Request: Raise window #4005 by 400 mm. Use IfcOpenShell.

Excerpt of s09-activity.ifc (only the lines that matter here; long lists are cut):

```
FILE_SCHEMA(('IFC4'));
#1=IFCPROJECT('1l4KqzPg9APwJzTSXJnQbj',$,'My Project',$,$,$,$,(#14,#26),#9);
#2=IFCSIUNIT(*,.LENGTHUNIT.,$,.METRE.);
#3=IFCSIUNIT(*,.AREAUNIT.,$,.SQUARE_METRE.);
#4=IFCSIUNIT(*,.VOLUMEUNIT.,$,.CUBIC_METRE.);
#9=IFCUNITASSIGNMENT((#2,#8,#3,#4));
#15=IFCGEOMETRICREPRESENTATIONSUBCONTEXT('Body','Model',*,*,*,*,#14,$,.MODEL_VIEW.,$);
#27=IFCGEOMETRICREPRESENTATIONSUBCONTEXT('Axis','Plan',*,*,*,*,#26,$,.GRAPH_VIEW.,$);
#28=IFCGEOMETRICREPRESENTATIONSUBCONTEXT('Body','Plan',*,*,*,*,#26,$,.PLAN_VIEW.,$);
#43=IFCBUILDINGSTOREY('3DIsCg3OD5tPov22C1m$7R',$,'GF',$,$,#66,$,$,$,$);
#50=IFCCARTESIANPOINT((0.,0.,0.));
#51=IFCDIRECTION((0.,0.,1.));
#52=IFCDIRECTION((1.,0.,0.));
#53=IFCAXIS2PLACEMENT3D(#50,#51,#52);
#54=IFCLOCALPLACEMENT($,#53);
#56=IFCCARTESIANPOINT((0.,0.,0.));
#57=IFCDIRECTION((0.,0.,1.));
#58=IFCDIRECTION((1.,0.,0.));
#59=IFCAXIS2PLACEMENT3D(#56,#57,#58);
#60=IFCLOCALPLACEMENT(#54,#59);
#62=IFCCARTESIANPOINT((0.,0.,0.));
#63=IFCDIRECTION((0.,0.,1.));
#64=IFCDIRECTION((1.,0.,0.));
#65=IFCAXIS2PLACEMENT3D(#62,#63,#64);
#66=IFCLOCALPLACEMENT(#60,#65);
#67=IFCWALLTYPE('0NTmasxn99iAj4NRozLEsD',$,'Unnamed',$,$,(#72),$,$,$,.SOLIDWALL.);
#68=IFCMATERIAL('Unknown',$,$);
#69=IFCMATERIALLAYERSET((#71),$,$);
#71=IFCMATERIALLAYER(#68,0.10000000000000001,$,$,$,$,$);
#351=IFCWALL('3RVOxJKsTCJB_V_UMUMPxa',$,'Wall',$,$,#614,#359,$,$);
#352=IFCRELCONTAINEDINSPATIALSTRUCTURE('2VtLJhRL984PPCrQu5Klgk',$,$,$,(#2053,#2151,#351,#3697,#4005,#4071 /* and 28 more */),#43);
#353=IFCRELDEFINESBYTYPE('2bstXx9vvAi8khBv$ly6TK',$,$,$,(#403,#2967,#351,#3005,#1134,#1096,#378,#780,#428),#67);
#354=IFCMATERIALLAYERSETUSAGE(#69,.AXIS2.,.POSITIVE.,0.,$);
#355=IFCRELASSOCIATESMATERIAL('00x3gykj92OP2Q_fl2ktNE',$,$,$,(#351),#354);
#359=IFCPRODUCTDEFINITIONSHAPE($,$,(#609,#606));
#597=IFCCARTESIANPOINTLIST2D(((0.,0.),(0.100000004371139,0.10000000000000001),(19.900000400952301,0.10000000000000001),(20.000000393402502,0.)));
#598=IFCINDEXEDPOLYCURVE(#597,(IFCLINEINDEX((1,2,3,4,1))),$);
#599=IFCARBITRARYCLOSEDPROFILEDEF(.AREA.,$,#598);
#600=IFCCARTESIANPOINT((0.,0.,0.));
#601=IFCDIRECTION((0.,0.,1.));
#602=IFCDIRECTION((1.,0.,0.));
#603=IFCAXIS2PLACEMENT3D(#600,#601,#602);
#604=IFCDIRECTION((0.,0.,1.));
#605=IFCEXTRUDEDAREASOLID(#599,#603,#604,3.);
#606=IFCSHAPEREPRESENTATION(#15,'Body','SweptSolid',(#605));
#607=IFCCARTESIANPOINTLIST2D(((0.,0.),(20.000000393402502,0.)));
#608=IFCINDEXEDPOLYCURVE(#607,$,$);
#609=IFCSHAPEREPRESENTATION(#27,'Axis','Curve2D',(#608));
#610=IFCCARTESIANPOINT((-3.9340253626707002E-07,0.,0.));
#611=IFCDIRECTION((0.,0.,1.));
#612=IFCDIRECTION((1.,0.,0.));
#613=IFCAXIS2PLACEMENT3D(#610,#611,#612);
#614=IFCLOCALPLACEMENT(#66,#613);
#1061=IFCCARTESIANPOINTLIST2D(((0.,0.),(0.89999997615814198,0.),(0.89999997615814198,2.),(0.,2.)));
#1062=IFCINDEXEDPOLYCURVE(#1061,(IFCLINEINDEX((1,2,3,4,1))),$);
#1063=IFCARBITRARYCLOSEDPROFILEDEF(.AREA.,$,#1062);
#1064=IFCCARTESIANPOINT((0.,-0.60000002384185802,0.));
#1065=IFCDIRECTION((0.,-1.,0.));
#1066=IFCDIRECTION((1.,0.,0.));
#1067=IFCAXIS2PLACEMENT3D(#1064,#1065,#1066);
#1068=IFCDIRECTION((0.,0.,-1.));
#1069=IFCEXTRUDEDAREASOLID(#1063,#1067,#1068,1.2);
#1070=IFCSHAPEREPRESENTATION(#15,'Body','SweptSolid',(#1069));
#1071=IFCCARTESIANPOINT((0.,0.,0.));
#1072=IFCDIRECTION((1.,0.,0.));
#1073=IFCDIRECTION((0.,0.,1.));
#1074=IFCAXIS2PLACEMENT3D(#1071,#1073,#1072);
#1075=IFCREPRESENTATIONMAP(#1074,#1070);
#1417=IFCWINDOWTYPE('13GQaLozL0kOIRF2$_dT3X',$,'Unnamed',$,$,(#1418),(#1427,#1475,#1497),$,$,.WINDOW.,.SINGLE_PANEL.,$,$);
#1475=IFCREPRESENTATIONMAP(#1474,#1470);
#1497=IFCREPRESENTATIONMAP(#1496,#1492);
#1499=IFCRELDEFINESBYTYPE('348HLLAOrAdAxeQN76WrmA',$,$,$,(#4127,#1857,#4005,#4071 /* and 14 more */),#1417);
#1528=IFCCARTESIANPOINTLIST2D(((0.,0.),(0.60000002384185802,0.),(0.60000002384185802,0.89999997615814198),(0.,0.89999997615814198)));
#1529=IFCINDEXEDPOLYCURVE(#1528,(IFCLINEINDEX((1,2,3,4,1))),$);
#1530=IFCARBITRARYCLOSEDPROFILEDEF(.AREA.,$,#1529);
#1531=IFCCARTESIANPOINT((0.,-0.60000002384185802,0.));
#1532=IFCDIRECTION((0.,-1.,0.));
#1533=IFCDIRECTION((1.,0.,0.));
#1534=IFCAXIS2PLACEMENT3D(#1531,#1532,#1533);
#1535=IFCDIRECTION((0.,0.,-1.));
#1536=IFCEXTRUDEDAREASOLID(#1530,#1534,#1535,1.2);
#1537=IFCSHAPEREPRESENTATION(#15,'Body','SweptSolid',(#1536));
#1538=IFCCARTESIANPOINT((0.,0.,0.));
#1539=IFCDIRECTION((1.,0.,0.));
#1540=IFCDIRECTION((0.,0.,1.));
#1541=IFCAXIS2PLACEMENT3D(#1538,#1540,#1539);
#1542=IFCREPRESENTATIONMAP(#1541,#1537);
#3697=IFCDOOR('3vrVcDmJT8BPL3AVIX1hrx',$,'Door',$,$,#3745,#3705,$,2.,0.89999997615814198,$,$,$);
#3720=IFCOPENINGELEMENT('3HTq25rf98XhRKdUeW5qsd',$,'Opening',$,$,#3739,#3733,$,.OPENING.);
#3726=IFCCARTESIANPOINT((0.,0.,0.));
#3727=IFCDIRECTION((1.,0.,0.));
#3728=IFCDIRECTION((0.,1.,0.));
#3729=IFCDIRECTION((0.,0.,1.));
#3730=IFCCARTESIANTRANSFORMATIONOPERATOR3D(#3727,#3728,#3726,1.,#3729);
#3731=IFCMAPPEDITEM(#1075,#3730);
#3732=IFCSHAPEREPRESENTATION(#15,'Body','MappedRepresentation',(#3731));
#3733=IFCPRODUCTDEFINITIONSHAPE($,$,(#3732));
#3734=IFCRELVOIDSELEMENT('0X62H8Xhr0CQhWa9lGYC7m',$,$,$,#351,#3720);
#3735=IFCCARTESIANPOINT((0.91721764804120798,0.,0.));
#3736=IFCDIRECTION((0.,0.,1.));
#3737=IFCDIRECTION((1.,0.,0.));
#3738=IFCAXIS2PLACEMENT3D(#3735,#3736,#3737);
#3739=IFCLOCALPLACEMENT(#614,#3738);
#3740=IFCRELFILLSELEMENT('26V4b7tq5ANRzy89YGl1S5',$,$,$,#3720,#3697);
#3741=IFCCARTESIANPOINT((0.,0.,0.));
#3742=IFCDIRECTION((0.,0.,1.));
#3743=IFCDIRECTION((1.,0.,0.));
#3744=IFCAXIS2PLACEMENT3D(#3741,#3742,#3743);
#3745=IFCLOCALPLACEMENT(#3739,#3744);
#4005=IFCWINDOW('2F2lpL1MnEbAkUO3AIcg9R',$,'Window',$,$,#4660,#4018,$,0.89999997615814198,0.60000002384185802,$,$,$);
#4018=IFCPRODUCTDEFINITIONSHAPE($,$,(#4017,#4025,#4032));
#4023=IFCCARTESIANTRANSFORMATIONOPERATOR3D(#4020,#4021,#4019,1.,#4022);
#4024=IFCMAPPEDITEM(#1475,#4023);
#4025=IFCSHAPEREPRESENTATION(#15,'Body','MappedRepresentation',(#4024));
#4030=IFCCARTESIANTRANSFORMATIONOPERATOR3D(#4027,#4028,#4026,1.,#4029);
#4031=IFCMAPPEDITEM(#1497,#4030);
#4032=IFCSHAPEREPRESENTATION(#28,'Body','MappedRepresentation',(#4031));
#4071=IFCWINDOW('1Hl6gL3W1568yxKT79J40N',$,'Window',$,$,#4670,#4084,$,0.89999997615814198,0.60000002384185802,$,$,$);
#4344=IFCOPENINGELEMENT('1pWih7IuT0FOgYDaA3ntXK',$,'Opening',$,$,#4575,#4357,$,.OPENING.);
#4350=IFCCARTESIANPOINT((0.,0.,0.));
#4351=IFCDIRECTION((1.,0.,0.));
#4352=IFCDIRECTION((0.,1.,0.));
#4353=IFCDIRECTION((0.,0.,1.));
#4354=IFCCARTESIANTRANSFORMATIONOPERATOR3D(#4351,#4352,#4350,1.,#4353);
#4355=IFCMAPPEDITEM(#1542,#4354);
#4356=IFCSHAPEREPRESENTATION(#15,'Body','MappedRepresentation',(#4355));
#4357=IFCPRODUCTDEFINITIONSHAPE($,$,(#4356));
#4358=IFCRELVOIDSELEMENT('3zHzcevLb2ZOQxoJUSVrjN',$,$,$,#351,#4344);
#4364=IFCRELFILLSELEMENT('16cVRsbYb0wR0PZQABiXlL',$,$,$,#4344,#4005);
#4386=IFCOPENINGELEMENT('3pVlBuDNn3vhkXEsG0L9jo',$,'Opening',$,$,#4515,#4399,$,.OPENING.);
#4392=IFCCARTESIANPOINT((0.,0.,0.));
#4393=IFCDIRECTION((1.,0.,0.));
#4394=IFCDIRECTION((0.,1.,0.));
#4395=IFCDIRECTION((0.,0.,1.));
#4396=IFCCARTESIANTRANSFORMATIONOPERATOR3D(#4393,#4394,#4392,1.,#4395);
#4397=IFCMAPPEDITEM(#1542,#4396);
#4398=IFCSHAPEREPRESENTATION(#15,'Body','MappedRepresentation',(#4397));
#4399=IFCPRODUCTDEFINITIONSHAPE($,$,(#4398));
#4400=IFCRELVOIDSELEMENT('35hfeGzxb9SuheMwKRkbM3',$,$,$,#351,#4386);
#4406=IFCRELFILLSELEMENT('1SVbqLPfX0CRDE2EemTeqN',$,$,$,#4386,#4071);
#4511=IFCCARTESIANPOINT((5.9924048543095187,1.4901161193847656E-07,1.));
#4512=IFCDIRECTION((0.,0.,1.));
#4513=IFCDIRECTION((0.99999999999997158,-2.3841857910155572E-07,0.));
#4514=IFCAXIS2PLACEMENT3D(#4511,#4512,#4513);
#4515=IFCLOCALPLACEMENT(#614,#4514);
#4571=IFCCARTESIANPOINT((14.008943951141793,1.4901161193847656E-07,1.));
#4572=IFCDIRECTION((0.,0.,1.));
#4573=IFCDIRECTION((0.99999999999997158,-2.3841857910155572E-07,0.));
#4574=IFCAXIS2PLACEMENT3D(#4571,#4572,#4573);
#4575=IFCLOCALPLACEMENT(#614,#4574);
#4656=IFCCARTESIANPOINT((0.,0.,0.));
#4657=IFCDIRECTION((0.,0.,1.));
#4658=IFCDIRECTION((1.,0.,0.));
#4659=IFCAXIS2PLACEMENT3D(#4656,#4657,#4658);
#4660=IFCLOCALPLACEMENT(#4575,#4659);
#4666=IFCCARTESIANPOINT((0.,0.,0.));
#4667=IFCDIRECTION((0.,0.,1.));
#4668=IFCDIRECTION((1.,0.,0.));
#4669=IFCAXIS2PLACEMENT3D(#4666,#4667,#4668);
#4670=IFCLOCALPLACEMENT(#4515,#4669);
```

```python
import numpy as np
import ifcopenshell
import ifcopenshell.api.geometry
import ifcopenshell.util.placement
import ifcopenshell.util.unit

model = ifcopenshell.open("s09-activity.ifc")
unit_scale = ifcopenshell.util.unit.calculate_unit_scale(model)

window = model.by_guid("2F2lpL1MnEbAkUO3AIcg9R")
opening = window.FillsVoids[0].RelatingOpeningElement
dz = 0.4 / unit_scale

shift = np.array([0.0, 0.0, dz])
# The window is placed relative to its opening, so it follows when the opening moves.
matrix = ifcopenshell.util.placement.get_local_placement(opening.ObjectPlacement)
matrix[:3, 3] += shift
ifcopenshell.api.geometry.edit_object_placement(
    model, product=opening, matrix=matrix, is_si=False, should_transform_children=True
)

print(f"moved by {dz * unit_scale:+.3f} m")

model.write("s09-activity_updated.ifc")
```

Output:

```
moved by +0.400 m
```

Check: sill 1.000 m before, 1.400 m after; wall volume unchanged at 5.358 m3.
